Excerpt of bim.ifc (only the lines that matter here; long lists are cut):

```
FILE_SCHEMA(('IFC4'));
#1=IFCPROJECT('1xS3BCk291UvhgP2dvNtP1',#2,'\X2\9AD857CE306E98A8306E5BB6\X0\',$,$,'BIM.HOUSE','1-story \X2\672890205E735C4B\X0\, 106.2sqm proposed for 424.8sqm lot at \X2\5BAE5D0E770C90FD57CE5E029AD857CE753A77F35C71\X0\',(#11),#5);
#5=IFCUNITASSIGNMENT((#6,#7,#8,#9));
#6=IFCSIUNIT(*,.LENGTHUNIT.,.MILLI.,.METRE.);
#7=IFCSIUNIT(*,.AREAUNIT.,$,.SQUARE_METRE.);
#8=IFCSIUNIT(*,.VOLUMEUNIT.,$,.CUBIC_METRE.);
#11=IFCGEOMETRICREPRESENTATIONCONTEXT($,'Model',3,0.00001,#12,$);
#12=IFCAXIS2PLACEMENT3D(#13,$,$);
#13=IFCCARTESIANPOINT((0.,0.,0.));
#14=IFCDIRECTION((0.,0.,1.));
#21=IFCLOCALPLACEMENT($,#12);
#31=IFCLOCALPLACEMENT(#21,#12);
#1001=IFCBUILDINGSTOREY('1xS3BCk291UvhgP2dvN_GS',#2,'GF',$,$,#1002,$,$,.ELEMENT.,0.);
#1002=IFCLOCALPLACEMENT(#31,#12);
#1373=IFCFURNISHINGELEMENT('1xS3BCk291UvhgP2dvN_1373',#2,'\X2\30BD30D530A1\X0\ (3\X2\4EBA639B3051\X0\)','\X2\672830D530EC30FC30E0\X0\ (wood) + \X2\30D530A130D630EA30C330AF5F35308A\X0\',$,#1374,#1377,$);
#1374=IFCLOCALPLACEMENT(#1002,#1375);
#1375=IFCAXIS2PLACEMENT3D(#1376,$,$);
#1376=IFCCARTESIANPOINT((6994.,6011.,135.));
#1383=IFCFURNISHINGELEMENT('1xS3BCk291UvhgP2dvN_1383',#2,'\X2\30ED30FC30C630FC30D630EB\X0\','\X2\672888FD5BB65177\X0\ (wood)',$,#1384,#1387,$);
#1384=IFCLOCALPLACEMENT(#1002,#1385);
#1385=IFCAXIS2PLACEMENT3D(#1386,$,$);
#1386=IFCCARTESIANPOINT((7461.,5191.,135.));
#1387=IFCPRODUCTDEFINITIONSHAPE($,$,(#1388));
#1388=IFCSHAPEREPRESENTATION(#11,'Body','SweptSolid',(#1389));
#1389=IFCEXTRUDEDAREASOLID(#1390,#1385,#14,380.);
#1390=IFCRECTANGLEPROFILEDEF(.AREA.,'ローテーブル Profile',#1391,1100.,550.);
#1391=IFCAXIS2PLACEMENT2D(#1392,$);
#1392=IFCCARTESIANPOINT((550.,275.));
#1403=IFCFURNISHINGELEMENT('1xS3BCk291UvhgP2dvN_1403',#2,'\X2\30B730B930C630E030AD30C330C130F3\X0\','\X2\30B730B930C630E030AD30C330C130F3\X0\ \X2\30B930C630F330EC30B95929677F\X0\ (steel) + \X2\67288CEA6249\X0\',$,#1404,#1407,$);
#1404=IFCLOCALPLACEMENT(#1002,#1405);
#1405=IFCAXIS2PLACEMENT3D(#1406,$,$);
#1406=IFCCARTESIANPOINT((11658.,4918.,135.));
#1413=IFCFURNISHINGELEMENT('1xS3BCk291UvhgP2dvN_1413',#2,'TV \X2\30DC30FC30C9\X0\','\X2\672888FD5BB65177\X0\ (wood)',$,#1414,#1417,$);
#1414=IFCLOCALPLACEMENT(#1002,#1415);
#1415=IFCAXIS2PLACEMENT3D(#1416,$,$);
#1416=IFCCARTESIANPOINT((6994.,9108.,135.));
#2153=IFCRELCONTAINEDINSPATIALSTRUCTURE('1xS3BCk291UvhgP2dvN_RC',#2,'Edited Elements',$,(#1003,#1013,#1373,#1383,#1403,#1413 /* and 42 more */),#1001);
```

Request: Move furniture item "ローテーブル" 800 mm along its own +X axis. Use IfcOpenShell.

```python
import ifcopenshell
import ifcopenshell.api.geometry
import ifcopenshell.util.placement
import ifcopenshell.util.unit

model = ifcopenshell.open("bim.ifc")
unit_scale = ifcopenshell.util.unit.calculate_unit_scale(model)

item = model.by_id(1383)
matrix = ifcopenshell.util.placement.get_local_placement(item.ObjectPlacement)
matrix[:3, 3] += matrix[:3, 0] * 0.8 / unit_scale
ifcopenshell.api.geometry.edit_object_placement(model, product=item, matrix=matrix, is_si=False)

print(ifcopenshell.util.placement.get_local_placement(item.ObjectPlacement).round(3) + 0.0)

model.write("bim_v2.ifc")
```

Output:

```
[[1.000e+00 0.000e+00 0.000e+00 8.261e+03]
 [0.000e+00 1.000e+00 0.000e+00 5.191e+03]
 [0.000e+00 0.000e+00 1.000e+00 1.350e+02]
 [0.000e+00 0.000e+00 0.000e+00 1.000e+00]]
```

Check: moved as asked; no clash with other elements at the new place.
